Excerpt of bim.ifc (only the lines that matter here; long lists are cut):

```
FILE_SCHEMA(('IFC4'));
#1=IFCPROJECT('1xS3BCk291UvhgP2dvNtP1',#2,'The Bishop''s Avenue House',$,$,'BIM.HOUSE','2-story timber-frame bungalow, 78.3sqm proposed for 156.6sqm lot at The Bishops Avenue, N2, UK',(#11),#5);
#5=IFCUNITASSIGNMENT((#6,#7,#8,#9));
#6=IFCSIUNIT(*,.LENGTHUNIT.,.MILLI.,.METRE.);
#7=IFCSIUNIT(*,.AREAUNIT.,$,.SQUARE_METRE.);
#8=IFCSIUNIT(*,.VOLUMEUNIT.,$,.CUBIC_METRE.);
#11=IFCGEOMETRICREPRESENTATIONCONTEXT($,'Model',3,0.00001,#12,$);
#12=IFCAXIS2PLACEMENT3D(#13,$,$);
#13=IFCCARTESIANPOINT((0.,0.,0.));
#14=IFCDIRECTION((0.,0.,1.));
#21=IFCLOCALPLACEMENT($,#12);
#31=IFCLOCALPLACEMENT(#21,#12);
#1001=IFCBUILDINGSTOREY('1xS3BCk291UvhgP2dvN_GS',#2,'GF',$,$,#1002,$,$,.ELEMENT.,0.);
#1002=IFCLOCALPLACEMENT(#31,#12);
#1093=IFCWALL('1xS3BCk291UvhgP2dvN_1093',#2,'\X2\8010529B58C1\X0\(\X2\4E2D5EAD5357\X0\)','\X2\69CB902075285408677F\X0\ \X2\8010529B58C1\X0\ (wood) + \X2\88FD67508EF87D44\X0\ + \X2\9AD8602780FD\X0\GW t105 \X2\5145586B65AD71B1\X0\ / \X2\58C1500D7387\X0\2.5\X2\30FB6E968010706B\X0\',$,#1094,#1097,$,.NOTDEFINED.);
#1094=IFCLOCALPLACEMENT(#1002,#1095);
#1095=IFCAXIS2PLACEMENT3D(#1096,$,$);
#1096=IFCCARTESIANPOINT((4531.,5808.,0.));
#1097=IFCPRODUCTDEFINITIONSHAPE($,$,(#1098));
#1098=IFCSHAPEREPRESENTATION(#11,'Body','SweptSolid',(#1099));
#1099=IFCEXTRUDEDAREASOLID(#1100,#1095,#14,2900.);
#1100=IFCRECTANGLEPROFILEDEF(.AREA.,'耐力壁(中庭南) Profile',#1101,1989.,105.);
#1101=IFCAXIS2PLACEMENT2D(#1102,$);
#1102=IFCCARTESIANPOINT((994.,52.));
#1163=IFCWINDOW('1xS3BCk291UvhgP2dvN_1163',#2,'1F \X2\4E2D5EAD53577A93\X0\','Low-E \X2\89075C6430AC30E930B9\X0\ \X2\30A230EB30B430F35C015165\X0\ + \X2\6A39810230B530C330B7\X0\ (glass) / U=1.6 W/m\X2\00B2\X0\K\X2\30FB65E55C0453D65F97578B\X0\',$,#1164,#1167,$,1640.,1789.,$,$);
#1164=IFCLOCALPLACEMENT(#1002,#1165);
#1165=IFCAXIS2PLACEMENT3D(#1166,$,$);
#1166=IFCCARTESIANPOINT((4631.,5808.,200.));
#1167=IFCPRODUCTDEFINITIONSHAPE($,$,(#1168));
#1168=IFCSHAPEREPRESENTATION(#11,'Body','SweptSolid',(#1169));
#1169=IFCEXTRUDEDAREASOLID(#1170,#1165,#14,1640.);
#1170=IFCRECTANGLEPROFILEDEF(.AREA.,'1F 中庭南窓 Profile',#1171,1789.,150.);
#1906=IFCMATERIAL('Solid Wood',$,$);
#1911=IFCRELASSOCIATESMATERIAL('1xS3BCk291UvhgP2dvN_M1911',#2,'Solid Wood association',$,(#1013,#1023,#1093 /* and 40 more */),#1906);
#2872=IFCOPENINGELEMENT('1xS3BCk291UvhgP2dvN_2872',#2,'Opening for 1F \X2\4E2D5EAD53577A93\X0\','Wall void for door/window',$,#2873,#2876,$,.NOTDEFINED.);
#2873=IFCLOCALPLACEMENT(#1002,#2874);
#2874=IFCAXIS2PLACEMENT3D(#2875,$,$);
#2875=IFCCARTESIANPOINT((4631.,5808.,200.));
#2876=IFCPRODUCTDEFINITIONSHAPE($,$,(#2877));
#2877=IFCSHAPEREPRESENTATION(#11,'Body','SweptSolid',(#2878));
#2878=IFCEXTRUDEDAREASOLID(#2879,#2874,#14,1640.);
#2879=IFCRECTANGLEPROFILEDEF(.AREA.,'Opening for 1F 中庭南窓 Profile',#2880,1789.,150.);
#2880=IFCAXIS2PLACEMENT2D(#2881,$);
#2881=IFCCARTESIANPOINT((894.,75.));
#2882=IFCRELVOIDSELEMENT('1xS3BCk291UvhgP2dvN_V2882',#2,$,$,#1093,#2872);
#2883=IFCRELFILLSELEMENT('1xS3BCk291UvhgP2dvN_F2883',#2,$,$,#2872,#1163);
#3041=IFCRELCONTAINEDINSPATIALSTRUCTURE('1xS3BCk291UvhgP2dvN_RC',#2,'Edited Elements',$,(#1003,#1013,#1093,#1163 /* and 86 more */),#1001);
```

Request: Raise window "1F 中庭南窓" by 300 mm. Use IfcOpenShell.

```python
import numpy as np
import ifcopenshell
import ifcopenshell.api.geometry
import ifcopenshell.util.placement
import ifcopenshell.util.unit

model = ifcopenshell.open("bim.ifc")
unit_scale = ifcopenshell.util.unit.calculate_unit_scale(model)

window = model.by_guid("1xS3BCk291UvhgP2dvN_1163")
opening = window.FillsVoids[0].RelatingOpeningElement
dz = 0.3 / unit_scale

shift = np.array([0.0, 0.0, dz])
# The window is not placed relative to its opening, so move both.
for product in (opening, window):
    matrix = ifcopenshell.util.placement.get_local_placement(product.ObjectPlacement)
    matrix[:3, 3] += shift
    ifcopenshell.api.geometry.edit_object_placement(model, product=product, matrix=matrix, is_si=False)

print(f"moved by {dz * unit_scale:+.3f} m")

model.write("bim_updated.ifc")
```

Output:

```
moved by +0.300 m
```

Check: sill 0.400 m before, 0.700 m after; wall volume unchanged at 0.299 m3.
